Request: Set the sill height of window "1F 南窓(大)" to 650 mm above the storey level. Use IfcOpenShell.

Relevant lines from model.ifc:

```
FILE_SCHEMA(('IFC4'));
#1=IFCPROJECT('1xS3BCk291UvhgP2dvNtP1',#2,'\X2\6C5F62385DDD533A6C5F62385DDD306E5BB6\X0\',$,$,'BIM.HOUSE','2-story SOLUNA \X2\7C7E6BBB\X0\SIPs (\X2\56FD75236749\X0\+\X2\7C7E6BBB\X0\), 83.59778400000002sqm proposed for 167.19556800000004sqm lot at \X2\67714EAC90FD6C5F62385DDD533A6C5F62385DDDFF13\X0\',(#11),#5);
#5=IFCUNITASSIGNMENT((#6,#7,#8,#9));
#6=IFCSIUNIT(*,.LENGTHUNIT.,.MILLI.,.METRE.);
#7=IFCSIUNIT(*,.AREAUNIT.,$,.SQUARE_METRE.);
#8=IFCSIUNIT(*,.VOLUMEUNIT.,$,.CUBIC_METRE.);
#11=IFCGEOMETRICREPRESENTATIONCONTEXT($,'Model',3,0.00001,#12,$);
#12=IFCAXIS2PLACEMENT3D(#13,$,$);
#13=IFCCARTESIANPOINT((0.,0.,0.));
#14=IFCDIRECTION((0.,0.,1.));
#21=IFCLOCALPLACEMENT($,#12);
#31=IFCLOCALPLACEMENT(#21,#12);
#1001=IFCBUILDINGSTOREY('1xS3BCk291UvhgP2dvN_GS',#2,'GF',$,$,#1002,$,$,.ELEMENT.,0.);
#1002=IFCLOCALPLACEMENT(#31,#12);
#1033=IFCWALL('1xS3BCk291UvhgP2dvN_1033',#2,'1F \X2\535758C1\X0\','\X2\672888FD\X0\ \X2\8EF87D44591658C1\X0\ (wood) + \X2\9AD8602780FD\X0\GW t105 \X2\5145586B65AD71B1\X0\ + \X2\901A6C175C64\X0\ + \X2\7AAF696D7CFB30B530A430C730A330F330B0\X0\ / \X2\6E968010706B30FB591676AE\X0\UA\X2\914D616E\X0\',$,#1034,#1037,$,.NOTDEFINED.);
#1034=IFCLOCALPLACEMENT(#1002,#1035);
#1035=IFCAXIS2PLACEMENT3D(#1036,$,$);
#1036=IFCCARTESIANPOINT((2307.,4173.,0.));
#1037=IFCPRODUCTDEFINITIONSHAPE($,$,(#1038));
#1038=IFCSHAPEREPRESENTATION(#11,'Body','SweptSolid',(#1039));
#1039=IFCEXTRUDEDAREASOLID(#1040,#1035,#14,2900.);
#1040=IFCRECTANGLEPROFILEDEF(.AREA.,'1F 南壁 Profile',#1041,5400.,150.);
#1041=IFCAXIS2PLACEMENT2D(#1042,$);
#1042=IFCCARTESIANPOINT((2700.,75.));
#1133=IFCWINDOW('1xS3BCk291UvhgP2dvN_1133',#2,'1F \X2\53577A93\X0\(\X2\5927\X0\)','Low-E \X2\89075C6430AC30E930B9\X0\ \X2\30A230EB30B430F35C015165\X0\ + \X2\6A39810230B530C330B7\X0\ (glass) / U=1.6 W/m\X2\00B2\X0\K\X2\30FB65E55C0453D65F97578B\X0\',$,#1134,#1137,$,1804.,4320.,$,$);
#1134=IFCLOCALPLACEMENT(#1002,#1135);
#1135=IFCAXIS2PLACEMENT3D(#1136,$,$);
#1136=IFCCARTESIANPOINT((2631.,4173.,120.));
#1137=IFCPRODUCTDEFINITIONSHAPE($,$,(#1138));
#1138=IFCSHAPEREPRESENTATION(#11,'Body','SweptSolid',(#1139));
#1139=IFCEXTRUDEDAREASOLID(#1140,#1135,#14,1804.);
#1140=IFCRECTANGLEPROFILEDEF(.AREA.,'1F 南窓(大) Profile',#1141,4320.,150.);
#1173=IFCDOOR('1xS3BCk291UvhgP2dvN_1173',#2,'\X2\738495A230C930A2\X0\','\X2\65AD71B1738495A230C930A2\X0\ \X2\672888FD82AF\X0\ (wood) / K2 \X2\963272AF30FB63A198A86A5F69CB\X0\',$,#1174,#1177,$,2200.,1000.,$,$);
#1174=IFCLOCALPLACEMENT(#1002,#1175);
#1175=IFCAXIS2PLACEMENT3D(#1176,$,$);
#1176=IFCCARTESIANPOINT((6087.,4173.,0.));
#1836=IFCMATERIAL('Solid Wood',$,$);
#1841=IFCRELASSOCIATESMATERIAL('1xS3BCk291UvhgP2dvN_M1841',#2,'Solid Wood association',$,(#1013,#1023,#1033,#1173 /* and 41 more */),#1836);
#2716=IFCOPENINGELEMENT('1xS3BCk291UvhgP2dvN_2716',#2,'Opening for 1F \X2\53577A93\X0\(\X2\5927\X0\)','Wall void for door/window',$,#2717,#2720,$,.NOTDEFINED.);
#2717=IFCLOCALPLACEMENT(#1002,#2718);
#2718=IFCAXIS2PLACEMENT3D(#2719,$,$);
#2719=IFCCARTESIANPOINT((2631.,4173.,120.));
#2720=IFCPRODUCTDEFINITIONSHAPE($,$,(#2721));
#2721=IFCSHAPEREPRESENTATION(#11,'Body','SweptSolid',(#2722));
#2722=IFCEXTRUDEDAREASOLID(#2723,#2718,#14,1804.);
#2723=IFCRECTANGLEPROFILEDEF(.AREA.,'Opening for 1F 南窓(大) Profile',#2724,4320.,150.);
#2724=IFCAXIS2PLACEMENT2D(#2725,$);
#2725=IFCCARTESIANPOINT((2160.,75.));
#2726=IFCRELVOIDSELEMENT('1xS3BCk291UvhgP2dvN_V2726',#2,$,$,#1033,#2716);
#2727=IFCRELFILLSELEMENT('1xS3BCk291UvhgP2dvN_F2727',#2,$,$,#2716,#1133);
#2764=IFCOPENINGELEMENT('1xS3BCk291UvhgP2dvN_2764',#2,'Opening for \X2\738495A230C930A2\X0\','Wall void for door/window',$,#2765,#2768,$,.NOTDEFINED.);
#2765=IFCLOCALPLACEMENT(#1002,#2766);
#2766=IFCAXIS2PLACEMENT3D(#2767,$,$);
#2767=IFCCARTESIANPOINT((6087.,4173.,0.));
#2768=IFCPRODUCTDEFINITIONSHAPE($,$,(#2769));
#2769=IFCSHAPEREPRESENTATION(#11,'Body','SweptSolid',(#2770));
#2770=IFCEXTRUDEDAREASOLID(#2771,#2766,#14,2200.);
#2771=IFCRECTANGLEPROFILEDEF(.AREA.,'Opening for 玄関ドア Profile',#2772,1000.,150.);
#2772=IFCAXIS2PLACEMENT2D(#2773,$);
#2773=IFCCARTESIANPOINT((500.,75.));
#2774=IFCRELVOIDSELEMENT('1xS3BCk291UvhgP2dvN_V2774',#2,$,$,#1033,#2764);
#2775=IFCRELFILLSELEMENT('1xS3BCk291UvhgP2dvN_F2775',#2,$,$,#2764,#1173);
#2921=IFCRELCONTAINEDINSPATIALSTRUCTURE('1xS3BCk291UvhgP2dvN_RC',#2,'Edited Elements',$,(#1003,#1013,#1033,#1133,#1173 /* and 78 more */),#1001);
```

```python
import numpy as np
import ifcopenshell
import ifcopenshell.api.geometry
import ifcopenshell.geom
import ifcopenshell.util.element
import ifcopenshell.util.placement
import ifcopenshell.util.shape
import ifcopenshell.util.unit

model = ifcopenshell.open("model.ifc")
unit_scale = ifcopenshell.util.unit.calculate_unit_scale(model)

window = model.by_guid("1xS3BCk291UvhgP2dvN_1133")
opening = window.FillsVoids[0].RelatingOpeningElement
storey = ifcopenshell.util.element.get_container(window, ifc_class="IfcBuildingStorey")
level = ifcopenshell.util.placement.get_local_placement(storey.ObjectPlacement)[2, 3]

# The opening's origin need not be at the sill, so measure its lowest point.
shape = ifcopenshell.geom.create_shape(ifcopenshell.geom.settings(), opening)
bottom = ifcopenshell.util.shape.get_shape_bottom_elevation(shape, shape.geometry) / unit_scale
dz = level + 0.65 / unit_scale - bottom

shift = np.array([0.0, 0.0, dz])
# The window is not placed relative to its opening, so move both.
for product in (opening, window):
    matrix = ifcopenshell.util.placement.get_local_placement(product.ObjectPlacement)
    matrix[:3, 3] += shift
    ifcopenshell.api.geometry.edit_object_placement(model, product=product, matrix=matrix, is_si=False)

print(f"moved by {dz * unit_scale:+.3f} m")

model.write("model_edited.ifc")
```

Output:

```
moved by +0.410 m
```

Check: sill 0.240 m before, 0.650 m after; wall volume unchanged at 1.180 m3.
